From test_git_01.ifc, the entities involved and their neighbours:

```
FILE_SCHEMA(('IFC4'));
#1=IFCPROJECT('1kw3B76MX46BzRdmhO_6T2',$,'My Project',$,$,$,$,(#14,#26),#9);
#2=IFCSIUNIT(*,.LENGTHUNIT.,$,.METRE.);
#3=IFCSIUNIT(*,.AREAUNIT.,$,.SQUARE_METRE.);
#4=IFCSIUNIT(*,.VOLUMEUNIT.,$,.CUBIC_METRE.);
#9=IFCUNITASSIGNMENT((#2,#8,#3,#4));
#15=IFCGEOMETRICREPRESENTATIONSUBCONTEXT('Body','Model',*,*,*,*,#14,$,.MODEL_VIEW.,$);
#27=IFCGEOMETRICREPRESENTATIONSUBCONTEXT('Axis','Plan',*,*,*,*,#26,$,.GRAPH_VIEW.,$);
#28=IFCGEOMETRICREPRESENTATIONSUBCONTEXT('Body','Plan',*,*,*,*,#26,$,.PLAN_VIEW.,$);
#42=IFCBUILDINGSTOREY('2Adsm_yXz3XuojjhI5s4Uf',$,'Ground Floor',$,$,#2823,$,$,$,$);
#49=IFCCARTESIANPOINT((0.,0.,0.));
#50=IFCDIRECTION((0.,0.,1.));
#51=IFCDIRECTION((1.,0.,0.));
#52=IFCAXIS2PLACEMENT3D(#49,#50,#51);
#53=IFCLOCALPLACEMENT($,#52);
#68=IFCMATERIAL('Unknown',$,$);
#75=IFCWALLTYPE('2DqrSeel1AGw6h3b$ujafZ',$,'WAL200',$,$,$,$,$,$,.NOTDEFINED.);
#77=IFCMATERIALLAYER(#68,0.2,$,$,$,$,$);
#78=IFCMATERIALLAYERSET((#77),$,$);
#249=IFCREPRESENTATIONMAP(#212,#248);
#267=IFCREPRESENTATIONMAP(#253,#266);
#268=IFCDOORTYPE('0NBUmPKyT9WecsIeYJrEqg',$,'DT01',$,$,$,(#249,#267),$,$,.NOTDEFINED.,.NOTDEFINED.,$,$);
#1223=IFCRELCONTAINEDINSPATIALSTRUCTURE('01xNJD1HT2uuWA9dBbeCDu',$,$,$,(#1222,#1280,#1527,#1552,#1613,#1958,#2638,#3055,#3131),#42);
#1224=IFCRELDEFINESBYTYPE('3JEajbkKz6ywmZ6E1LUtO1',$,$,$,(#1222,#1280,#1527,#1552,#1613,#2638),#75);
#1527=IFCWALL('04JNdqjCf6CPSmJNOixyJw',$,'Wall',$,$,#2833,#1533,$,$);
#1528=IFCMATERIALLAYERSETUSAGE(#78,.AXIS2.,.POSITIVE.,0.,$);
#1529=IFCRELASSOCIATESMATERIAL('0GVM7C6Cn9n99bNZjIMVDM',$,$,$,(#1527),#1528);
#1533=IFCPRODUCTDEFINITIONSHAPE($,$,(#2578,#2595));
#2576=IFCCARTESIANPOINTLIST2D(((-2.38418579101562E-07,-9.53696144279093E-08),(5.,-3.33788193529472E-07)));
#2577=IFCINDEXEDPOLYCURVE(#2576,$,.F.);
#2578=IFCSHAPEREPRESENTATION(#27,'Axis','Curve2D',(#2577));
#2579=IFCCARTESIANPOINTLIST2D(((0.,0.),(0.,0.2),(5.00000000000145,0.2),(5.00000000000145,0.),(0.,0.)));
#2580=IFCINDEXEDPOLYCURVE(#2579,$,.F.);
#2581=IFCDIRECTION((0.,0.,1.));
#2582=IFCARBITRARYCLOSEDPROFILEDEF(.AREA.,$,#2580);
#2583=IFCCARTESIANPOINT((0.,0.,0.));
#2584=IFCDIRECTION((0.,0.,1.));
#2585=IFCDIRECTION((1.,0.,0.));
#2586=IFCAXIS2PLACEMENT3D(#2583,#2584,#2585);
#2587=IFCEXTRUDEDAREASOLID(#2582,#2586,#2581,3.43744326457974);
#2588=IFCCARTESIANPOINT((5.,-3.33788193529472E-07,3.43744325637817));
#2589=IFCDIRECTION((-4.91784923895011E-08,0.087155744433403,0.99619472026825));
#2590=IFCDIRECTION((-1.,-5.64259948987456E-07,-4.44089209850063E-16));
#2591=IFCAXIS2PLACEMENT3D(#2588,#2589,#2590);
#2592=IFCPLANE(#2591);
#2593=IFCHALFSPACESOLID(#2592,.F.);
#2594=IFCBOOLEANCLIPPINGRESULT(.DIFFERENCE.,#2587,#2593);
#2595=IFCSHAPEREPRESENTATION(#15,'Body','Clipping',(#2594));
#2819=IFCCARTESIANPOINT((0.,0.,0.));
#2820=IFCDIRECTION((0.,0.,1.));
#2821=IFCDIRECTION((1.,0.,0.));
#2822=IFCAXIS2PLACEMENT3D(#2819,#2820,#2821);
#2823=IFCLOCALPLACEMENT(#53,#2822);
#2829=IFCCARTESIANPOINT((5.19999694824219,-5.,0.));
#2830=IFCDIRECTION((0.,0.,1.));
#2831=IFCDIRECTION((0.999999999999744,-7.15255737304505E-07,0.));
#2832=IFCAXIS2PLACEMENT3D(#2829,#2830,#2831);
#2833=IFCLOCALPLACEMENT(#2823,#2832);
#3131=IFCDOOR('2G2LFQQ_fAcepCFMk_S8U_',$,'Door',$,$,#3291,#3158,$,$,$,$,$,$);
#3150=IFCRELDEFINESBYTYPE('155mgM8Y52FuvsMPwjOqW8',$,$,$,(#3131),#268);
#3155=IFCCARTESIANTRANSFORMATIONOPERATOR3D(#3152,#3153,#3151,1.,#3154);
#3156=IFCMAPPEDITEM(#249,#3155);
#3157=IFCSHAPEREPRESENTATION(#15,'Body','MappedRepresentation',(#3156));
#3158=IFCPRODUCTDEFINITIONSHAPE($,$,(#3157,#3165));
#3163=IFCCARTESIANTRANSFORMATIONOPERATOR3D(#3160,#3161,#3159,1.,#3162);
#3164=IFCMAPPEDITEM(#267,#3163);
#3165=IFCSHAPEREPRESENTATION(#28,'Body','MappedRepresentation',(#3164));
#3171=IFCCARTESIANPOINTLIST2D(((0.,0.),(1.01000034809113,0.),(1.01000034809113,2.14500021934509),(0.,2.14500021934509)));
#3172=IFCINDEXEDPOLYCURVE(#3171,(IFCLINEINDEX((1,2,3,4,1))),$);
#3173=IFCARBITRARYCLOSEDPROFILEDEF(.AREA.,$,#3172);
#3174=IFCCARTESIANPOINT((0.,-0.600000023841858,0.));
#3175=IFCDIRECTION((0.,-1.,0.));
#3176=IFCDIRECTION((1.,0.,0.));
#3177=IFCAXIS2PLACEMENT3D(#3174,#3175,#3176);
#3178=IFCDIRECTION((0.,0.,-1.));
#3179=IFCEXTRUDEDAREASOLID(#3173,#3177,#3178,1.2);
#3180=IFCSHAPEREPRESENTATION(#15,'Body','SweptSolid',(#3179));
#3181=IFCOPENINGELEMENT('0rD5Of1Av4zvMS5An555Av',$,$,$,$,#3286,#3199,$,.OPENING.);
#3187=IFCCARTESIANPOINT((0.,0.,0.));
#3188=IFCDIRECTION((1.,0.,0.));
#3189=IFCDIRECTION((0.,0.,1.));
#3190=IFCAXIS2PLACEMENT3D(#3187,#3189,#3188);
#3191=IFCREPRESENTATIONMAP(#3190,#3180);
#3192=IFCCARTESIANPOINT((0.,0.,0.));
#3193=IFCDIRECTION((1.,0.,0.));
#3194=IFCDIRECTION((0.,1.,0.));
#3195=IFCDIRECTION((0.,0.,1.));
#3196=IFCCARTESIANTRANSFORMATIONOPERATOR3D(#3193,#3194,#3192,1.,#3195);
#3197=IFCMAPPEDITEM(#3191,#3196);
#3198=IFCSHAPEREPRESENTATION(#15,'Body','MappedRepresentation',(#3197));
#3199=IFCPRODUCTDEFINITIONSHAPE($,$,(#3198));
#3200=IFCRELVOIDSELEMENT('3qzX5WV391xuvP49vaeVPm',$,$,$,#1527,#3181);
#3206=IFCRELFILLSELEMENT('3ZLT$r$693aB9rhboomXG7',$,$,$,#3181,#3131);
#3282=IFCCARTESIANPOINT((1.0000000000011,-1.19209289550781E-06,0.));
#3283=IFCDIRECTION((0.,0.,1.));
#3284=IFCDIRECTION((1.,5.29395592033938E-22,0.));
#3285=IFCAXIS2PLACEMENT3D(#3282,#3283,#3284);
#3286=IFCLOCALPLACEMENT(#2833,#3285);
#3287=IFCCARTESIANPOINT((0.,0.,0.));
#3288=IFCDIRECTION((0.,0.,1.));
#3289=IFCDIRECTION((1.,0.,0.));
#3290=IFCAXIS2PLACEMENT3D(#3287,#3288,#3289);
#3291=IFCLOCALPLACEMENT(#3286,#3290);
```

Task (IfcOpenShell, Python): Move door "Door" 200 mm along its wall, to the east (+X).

```python
import ifcopenshell
import ifcopenshell.api.geometry
import ifcopenshell.util.placement

model = ifcopenshell.open("test_git_01.ifc")

door = model.by_id(3131)
opening = door.FillsVoids[0].RelatingOpeningElement
wall = opening.VoidsElements[0].RelatingBuildingElement

wall_matrix = ifcopenshell.util.placement.get_local_placement(wall.ObjectPlacement)
shift = wall_matrix[:3, 0] * 0.2
before = ifcopenshell.util.placement.get_local_placement(door.ObjectPlacement)[:3, 3].copy()

# The door is placed relative to its opening, so it follows when the opening moves.
matrix = ifcopenshell.util.placement.get_local_placement(opening.ObjectPlacement)
matrix[:3, 3] += shift
ifcopenshell.api.geometry.edit_object_placement(
    model, product=opening, matrix=matrix, is_si=False, should_transform_children=True
)

after = ifcopenshell.util.placement.get_local_placement(door.ObjectPlacement)[:3, 3]
print("door moved by", (after - before).round(3) + 0.0)

model.write("test_git_01_v2.ifc")
```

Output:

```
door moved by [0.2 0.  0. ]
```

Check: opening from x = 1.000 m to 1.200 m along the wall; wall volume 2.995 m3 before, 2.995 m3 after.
